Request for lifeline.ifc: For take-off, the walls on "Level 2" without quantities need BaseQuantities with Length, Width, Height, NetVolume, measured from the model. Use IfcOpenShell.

First a look at what the model holds.

```python
import ifcopenshell
import ifcopenshell.util.element
import ifcopenshell.util.unit

model = ifcopenshell.open("lifeline.ifc")
print(model.schema)
for unit_type in ("LENGTHUNIT", "AREAUNIT", "VOLUMEUNIT"):
    print(unit_type, ifcopenshell.util.unit.calculate_unit_scale(model, unit_type))
storey = next(s for s in model.by_type("IfcBuildingStorey") if s.Name == "Level 2")
walls = [e for e in ifcopenshell.util.element.get_decomposition(storey) if e.is_a("IfcWall")]
for e in sorted(walls, key=lambda e: e.id()):
    print(e.id(), e.is_a(), e.Name, list(ifcopenshell.util.element.get_psets(e, qtos_only=True)), sep=" | ")
```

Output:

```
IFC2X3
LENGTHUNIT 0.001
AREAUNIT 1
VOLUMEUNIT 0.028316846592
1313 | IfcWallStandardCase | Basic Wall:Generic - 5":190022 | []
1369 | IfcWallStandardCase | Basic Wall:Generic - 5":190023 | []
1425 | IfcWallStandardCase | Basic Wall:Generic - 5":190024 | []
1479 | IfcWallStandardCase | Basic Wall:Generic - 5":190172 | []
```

```python
import ifcopenshell
import ifcopenshell.api.pset
import ifcopenshell.geom
import ifcopenshell.util.element
import ifcopenshell.util.shape
import ifcopenshell.util.unit

model = ifcopenshell.open("lifeline.ifc")
unit_scale = ifcopenshell.util.unit.calculate_unit_scale(model)
volume_scale = ifcopenshell.util.unit.calculate_unit_scale(model, "VOLUMEUNIT")
settings = ifcopenshell.geom.settings()

storey = next(s for s in model.by_type("IfcBuildingStorey") if s.Name == "Level 2")
walls = [e for e in ifcopenshell.util.element.get_decomposition(storey) if e.is_a("IfcWall")]

for e in sorted(walls, key=lambda e: e.id()):
    if ifcopenshell.util.element.get_psets(e, qtos_only=True, should_inherit=False):
        continue
    # Geometry comes back in metres, in the element's own axes.
    shape = ifcopenshell.geom.create_shape(settings, e)
    values = {
        "Length": ifcopenshell.util.shape.get_x(shape.geometry) / unit_scale,
        "Width": ifcopenshell.util.shape.get_y(shape.geometry) / unit_scale,
        "Height": ifcopenshell.util.shape.get_z(shape.geometry) / unit_scale,
        "NetVolume": ifcopenshell.util.shape.get_volume(shape.geometry) / volume_scale,
    }
    qto = ifcopenshell.api.pset.add_qto(model, product=e, name="BaseQuantities")
    ifcopenshell.api.pset.edit_qto(model, qto=qto, properties=values)
    print(e.id(), {k: round(v, 3) for k, v in values.items()})

model.write("lifeline_rev.ifc")
```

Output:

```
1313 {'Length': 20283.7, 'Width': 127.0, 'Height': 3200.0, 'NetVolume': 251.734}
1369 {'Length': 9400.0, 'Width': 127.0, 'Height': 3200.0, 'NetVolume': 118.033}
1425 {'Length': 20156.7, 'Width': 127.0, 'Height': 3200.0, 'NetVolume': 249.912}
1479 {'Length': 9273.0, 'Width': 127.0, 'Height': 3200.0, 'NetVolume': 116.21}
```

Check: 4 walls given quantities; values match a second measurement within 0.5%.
